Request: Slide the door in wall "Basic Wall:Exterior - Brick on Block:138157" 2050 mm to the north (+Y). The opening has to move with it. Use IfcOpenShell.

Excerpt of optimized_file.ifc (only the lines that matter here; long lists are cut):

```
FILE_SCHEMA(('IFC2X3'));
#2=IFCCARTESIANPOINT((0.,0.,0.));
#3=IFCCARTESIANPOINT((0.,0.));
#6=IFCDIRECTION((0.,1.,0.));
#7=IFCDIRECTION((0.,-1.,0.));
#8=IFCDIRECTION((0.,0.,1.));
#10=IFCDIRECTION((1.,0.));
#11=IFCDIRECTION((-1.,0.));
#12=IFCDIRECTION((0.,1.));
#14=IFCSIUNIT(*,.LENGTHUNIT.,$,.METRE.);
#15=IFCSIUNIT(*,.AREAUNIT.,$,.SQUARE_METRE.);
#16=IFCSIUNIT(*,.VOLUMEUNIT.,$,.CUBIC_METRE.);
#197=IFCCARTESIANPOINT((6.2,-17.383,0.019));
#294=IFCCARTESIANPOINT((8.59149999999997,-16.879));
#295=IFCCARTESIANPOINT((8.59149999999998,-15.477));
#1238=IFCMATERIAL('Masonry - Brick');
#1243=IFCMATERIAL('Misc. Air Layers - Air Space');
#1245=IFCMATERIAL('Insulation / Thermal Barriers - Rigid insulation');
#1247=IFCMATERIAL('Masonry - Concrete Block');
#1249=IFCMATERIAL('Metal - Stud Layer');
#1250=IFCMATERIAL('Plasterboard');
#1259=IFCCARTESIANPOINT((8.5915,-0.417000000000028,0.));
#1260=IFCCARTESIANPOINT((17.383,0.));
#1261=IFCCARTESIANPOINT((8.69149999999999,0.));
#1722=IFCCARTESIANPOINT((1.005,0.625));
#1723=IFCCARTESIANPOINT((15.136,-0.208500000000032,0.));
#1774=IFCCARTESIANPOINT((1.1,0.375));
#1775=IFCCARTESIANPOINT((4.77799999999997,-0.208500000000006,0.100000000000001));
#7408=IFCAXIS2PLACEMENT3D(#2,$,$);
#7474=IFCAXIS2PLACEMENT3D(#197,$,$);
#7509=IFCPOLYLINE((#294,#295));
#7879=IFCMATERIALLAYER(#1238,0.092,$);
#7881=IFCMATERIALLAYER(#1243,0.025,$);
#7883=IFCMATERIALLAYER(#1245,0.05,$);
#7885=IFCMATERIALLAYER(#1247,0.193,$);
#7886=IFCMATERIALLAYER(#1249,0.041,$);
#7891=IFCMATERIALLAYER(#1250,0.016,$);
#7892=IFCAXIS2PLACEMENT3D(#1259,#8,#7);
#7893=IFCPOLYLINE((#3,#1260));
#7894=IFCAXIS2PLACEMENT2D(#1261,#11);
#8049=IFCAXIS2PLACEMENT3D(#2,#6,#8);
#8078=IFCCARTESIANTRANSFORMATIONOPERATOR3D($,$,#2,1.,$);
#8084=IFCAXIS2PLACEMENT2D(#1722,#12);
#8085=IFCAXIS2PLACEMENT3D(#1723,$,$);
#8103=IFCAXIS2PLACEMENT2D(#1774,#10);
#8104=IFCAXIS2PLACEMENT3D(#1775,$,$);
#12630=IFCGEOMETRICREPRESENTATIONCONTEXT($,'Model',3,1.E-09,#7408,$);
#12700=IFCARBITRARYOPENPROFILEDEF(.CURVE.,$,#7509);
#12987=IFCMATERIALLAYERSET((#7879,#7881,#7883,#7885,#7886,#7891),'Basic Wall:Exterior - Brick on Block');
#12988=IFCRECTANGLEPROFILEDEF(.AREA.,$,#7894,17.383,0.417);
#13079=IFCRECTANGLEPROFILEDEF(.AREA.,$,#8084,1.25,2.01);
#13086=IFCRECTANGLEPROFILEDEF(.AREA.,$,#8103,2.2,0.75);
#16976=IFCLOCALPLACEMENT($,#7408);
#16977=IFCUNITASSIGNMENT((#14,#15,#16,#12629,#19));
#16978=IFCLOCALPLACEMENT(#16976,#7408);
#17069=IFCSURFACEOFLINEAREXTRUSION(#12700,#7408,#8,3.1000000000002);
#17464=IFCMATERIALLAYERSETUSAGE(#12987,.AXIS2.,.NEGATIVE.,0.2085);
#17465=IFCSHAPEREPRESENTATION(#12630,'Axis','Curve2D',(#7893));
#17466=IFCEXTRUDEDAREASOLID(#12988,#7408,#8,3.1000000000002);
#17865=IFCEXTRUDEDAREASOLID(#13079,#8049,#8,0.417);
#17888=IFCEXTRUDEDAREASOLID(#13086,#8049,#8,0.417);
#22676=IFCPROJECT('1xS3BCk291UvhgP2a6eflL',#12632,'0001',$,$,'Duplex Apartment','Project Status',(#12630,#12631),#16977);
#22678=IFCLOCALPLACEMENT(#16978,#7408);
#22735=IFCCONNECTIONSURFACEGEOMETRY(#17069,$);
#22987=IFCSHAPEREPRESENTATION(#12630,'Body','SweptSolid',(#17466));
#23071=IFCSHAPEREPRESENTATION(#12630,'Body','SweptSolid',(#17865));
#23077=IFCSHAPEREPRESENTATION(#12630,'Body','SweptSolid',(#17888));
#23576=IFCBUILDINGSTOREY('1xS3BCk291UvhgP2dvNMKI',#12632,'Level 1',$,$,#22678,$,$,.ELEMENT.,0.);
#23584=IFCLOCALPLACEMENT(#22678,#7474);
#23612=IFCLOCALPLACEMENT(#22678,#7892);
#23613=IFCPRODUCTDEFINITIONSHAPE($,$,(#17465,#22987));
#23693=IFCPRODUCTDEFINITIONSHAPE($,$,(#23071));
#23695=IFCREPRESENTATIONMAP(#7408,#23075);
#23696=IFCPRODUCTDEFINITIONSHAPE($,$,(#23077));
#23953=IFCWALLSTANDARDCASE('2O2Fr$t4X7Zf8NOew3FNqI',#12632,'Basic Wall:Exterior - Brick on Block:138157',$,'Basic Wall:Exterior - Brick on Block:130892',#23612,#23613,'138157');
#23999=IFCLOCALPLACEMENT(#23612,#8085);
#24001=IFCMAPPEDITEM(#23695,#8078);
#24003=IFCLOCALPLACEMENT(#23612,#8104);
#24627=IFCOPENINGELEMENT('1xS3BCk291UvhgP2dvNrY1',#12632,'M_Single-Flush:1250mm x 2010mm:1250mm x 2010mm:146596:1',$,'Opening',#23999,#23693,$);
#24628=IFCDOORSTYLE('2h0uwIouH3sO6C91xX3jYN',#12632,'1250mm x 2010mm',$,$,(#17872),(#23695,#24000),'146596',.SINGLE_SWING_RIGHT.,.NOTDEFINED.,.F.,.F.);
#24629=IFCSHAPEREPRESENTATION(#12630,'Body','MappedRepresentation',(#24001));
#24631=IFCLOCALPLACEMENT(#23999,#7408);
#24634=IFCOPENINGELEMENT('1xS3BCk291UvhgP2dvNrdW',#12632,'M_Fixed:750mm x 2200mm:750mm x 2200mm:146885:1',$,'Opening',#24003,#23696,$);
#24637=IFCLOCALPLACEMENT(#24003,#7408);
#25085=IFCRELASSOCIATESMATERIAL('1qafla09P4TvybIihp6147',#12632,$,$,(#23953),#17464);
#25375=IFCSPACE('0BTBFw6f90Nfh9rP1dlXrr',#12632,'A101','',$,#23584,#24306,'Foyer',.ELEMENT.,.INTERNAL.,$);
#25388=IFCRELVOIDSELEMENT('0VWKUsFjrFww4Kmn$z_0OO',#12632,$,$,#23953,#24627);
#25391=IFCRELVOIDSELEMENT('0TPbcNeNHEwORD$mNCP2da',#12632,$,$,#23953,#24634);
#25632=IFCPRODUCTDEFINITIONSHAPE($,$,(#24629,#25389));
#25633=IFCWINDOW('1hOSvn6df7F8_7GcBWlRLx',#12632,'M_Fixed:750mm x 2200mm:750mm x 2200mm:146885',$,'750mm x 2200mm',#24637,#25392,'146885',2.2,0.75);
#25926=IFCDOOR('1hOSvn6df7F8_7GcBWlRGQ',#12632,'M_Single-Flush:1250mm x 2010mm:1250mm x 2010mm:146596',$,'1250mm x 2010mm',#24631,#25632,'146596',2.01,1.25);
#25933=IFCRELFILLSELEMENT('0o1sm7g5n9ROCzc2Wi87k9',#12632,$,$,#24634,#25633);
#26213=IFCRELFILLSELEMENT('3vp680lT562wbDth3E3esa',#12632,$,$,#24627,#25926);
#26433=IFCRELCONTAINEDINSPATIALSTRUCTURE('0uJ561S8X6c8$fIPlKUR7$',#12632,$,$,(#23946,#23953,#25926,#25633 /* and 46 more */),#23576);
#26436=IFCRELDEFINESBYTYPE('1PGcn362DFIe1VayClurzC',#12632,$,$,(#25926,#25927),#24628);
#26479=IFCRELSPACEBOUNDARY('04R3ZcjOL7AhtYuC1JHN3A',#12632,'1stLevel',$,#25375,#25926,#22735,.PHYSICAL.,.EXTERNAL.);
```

```python
import numpy as np
import ifcopenshell
import ifcopenshell.api.geometry
import ifcopenshell.util.placement
import ifcopenshell.util.unit

model = ifcopenshell.open("optimized_file.ifc")
unit_scale = ifcopenshell.util.unit.calculate_unit_scale(model)

door = model.by_id(25926)
opening = door.FillsVoids[0].RelatingOpeningElement
wall = opening.VoidsElements[0].RelatingBuildingElement

wall_matrix = ifcopenshell.util.placement.get_local_placement(wall.ObjectPlacement)
shift = wall_matrix[:3, 0] * -2.05 / unit_scale
before = ifcopenshell.util.placement.get_local_placement(door.ObjectPlacement)[:3, 3].copy()

# The door is placed relative to its opening, so it follows when the opening moves.
matrix = ifcopenshell.util.placement.get_local_placement(opening.ObjectPlacement)
matrix[:3, 3] += shift
ifcopenshell.api.geometry.edit_object_placement(
    model, product=opening, matrix=matrix, is_si=False, should_transform_children=True
)

# Space boundary surfaces are stored in each space's coordinates; move them too.
for rel in door.ProvidesBoundaries:
    if not rel.ConnectionGeometry:
        continue
    surface = rel.ConnectionGeometry.SurfaceOnRelatingElement
    space_matrix = ifcopenshell.util.placement.get_local_placement(rel.RelatingSpace.ObjectPlacement)
    point = np.array(surface.Position.Location.Coordinates) + space_matrix[:3, :3].T @ shift
    surface.Position = model.createIfcAxis2Placement3D(
        model.createIfcCartesianPoint(point.tolist()), surface.Position.Axis, surface.Position.RefDirection
    )

after = ifcopenshell.util.placement.get_local_placement(door.ObjectPlacement)[:3, 3]
print("door moved by", (after - before).round(3) + 0.0)

model.write("optimized_file_edited.ifc")
```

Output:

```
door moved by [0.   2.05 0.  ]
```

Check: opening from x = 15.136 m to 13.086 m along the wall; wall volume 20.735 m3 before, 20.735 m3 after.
